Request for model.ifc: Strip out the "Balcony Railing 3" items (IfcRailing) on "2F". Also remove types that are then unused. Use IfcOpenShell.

First a look at what the model holds.

```python
import ifcopenshell
import ifcopenshell.util.element

model = ifcopenshell.open("model.ifc")
print(model.schema)
storey = next(s for s in model.by_type("IfcBuildingStorey") if s.Name == "2F")
railings = [e for e in ifcopenshell.util.element.get_decomposition(storey) if e.is_a("IfcRailing")]
seen = {}
for e in railings:
    element_type = ifcopenshell.util.element.get_type(e)
    name = element_type.Name if element_type not in (None, e) else None
    seen[name] = seen.get(name, 0) + 1
for name, count in sorted(seen.items(), key=str):
    print(count, "x", name)
```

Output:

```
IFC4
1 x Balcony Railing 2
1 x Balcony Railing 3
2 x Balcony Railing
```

```python
import ifcopenshell
import ifcopenshell.api.root
import ifcopenshell.util.element

model = ifcopenshell.open("model.ifc")

storey = next(s for s in model.by_type("IfcBuildingStorey") if s.Name == "2F")
railings = [e for e in ifcopenshell.util.element.get_decomposition(storey) if e.is_a("IfcRailing")]
targets = [e for e in railings if (t := ifcopenshell.util.element.get_type(e)) not in (None, e) and t.Name == "Balcony Railing 3"]
types = {ifcopenshell.util.element.get_type(e) for e in targets} - {None, *targets}

for e in targets:
    ifcopenshell.api.root.remove_product(model, product=e)
print(len(targets), "removed")

unused = [t for t in types if not ifcopenshell.util.element.get_types(t)]
for t in unused:
    ifcopenshell.api.root.remove_product(model, product=t)
print(len(unused), "unused types removed")

model.write("model_v2.ifc")
```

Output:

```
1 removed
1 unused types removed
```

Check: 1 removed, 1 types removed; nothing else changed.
